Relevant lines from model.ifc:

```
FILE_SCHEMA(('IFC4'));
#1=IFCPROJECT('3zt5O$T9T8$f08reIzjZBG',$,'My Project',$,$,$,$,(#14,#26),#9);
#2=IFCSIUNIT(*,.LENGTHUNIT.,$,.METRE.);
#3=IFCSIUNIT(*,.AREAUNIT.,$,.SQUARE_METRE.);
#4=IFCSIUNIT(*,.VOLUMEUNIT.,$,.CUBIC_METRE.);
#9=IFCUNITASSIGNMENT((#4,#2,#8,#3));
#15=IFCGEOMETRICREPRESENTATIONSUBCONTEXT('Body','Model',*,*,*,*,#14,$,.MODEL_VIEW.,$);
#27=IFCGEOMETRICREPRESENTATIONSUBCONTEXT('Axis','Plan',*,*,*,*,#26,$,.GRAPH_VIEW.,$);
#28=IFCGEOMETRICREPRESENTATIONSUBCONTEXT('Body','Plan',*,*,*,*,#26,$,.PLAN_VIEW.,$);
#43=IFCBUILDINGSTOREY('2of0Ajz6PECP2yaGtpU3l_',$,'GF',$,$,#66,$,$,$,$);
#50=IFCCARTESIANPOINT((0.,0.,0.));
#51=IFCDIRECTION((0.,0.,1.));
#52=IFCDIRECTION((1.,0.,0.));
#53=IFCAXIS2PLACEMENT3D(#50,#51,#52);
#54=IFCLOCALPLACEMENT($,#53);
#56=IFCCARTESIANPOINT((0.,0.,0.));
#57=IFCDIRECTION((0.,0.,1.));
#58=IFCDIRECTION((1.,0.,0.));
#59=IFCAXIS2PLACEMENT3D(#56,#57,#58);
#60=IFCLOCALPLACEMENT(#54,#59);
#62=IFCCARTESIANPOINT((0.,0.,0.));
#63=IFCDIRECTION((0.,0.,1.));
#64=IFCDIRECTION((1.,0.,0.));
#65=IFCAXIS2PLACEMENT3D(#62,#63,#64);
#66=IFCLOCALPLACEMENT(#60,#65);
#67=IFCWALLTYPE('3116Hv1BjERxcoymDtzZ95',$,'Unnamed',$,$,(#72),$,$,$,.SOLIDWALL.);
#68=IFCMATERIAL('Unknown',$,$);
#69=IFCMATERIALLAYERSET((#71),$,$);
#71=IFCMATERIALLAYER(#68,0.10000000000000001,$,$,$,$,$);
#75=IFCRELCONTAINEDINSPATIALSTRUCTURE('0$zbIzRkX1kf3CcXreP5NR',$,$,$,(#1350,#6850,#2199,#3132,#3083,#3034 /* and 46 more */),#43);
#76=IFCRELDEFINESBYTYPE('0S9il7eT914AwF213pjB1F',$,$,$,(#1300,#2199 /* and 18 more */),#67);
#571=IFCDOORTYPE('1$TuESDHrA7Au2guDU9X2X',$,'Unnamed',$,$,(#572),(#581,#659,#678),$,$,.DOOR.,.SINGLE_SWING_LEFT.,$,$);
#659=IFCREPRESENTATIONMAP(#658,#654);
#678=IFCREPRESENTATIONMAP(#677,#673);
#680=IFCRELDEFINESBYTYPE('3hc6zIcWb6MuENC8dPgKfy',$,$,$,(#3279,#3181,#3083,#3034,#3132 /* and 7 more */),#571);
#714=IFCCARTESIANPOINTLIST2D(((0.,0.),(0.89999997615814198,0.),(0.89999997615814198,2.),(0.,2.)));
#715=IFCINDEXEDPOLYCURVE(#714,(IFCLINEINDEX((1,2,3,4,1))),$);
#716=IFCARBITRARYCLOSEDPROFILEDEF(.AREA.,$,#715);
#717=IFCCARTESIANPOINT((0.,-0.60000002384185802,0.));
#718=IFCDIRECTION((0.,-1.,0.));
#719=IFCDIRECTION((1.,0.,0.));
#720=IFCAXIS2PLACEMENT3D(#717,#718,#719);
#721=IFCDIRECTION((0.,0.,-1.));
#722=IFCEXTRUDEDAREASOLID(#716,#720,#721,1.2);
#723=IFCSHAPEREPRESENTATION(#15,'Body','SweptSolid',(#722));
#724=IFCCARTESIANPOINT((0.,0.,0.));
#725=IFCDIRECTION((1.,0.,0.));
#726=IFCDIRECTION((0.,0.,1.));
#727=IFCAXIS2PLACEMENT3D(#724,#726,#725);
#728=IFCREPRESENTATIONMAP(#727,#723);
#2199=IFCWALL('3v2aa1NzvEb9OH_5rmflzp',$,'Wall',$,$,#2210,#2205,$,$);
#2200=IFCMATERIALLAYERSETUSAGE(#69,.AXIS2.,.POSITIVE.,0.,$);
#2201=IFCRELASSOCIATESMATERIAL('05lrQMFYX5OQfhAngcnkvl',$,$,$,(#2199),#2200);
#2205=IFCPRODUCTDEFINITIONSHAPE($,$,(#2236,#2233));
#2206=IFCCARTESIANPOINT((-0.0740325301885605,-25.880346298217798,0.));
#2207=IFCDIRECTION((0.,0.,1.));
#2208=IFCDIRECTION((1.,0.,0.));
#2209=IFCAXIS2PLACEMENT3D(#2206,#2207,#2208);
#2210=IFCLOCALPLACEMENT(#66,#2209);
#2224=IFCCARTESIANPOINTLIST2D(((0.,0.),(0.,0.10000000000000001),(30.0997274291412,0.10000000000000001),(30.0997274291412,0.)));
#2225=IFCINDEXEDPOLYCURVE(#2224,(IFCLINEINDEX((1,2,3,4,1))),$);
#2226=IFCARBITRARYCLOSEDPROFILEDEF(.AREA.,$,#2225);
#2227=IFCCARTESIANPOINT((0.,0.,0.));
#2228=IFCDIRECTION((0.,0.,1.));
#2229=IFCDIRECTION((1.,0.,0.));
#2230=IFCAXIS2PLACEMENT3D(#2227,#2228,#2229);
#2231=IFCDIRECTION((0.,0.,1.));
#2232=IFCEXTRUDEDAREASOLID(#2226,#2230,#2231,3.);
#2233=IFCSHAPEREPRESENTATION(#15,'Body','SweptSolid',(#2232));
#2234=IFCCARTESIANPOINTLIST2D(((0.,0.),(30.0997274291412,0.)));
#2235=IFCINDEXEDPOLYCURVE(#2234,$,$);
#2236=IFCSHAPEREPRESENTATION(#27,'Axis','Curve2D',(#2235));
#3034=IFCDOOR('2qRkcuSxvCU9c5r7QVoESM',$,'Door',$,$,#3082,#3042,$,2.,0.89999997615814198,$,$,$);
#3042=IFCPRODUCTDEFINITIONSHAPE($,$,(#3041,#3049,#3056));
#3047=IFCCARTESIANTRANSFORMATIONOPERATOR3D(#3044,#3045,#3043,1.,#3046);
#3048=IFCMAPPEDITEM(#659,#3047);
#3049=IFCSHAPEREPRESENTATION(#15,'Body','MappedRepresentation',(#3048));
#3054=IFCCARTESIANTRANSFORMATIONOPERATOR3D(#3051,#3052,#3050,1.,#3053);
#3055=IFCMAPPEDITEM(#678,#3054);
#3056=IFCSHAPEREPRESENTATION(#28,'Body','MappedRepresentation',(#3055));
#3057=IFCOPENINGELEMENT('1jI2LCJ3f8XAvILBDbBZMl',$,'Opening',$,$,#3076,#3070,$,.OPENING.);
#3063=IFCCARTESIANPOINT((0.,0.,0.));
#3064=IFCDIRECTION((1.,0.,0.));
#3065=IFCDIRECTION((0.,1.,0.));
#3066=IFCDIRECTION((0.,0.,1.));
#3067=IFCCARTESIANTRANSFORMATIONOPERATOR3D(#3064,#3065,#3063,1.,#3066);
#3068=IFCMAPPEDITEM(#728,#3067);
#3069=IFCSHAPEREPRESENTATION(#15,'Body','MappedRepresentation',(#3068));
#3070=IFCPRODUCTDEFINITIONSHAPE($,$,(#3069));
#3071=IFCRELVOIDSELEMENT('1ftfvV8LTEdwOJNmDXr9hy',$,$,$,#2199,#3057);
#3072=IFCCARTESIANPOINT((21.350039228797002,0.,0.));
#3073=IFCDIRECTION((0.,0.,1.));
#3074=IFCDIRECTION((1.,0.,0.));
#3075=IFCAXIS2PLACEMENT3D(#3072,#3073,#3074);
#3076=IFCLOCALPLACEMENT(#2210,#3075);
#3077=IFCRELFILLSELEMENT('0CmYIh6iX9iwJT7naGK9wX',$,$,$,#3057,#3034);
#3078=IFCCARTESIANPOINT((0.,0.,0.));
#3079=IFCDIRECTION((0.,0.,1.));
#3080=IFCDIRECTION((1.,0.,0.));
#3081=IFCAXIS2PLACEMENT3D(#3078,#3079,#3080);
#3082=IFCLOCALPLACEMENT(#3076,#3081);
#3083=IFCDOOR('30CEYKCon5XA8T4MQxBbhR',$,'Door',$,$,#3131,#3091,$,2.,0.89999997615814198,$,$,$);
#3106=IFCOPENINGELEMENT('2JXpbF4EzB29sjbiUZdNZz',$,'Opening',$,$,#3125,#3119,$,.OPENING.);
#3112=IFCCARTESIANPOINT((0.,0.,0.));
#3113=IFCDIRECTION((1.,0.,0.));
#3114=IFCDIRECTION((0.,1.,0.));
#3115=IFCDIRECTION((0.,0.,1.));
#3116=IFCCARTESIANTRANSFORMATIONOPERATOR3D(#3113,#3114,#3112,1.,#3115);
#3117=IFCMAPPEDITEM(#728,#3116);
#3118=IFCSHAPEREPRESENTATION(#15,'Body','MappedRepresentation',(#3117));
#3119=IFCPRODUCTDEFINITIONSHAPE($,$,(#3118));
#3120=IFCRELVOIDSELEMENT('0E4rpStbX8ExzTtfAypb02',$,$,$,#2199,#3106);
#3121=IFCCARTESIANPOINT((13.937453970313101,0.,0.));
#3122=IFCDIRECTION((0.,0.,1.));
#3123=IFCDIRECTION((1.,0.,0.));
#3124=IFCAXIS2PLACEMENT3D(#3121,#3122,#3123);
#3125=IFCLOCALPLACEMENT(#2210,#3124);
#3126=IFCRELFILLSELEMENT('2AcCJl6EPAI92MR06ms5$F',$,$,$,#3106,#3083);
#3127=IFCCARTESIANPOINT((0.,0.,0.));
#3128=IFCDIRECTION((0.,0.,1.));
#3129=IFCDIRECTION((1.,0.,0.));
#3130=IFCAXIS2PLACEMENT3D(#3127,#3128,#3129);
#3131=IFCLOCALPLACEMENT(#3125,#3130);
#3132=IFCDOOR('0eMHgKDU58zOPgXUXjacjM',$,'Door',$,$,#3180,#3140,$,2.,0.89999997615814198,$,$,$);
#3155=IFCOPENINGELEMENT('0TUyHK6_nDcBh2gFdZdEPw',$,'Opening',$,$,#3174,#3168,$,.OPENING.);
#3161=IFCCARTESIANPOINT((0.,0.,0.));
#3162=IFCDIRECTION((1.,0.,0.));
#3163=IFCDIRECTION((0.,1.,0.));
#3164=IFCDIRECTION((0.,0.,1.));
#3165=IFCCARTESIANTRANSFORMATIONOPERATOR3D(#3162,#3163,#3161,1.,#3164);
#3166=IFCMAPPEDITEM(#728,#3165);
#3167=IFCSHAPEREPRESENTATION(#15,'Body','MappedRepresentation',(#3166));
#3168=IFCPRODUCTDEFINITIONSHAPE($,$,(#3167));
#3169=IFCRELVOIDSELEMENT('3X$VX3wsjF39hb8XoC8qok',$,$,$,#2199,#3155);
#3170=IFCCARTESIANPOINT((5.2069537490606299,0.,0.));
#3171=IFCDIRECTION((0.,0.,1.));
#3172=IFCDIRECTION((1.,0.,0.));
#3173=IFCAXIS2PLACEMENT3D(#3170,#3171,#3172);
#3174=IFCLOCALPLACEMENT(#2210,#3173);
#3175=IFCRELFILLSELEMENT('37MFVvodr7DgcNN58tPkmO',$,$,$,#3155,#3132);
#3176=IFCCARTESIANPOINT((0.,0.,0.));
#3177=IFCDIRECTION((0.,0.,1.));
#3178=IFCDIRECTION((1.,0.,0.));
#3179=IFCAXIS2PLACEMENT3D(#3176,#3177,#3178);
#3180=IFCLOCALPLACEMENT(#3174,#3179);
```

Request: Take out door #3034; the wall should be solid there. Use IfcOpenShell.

```python
import ifcopenshell
import ifcopenshell.api.feature
import ifcopenshell.api.root
import ifcopenshell.geom
import ifcopenshell.util.shape

model = ifcopenshell.open("model.ifc")
settings = ifcopenshell.geom.settings()


def volume(element):
    """Net volume in cubic metres, openings subtracted."""
    shape = ifcopenshell.geom.create_shape(settings, element)
    return ifcopenshell.util.shape.get_volume(shape.geometry)


door = model.by_guid("2qRkcuSxvCU9c5r7QVoESM")
opening = door.FillsVoids[0].RelatingOpeningElement
wall = opening.VoidsElements[0].RelatingBuildingElement
before = volume(wall)

ifcopenshell.api.root.remove_product(model, product=door)
ifcopenshell.api.feature.remove_feature(model, feature=opening)

after = volume(wall)

print(f"wall volume {before:.3f} -> {after:.3f} m3")

model.write("model_edited.ifc")
```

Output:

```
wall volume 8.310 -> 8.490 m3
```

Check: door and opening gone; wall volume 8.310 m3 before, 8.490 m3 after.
